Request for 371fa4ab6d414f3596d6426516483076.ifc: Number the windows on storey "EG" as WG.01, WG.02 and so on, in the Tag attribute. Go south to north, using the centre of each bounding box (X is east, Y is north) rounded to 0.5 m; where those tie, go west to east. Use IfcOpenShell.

First a look at what the model holds.

```python
import ifcopenshell
import ifcopenshell.util.element
import ifcopenshell.util.placement

model = ifcopenshell.open("371fa4ab6d414f3596d6426516483076.ifc")
print(model.schema)
storey = next(s for s in model.by_type("IfcBuildingStorey") if s.Name == "EG")
windows = [e for e in ifcopenshell.util.element.get_decomposition(storey) if e.is_a("IfcWindow")]
for e in sorted(windows, key=lambda e: e.id()):
    origin = ifcopenshell.util.placement.get_local_placement(e.ObjectPlacement)[:3, 3]
    print(e.id(), e.Tag, e.Name, origin.round(2) + 0.0, sep=" | ")
```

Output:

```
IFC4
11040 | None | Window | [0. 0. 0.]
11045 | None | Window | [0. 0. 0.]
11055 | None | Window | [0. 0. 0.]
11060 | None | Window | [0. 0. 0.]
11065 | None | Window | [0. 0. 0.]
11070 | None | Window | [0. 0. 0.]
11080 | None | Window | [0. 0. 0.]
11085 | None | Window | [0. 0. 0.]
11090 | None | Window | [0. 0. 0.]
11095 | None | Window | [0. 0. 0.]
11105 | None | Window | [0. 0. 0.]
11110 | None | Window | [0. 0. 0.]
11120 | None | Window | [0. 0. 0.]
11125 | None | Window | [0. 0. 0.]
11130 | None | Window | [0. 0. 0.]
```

```python
import ifcopenshell
import ifcopenshell.geom
import ifcopenshell.util.element
import ifcopenshell.util.shape

model = ifcopenshell.open("371fa4ab6d414f3596d6426516483076.ifc")
settings = ifcopenshell.geom.settings()
settings.set("use-world-coords", True)


def centre(element):
    shape = ifcopenshell.geom.create_shape(settings, element)
    return ifcopenshell.util.shape.get_bbox_centroid(shape.geometry)


storey = next(s for s in model.by_type("IfcBuildingStorey") if s.Name == "EG")
windows = [e for e in ifcopenshell.util.element.get_decomposition(storey) if e.is_a("IfcWindow")]

# Insertion points can sit at a corner or the storey origin, so sort by the geometry (in metres).
centres = {e: centre(e) for e in windows}
windows.sort(key=lambda e: (round(centres[e][1] / 0.5), centres[e][0]))

for i, e in enumerate(windows, start=1):
    number = f"WG.{i:02d}"
    e.Tag = number
    print(e.id(), number)

model.write("371fa4ab6d414f3596d6426516483076_rev.ifc")
```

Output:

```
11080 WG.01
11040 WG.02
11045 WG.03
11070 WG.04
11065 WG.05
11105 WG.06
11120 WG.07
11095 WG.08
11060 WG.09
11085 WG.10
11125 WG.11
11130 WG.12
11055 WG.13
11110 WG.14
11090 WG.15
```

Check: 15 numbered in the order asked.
